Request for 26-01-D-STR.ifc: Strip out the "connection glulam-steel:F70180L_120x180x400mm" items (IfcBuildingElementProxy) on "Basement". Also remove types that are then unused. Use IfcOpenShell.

First a look at what the model holds.

```python
import ifcopenshell
import ifcopenshell.util.element

model = ifcopenshell.open("26-01-D-STR.ifc")
print(model.schema)
storey = next(s for s in model.by_type("IfcBuildingStorey") if s.Name == "Basement")
proxies = [e for e in ifcopenshell.util.element.get_decomposition(storey) if e.is_a("IfcBuildingElementProxy")]
seen = {}
for e in proxies:
    element_type = ifcopenshell.util.element.get_type(e)
    name = element_type.Name if element_type not in (None, e) else None
    seen[name] = seen.get(name, 0) + 1
for name, count in sorted(seen.items(), key=str):
    print(count, "x", name)
```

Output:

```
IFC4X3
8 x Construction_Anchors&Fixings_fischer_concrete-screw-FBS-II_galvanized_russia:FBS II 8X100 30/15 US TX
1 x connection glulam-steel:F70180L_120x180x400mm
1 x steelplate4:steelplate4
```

```python
import ifcopenshell
import ifcopenshell.api.root
import ifcopenshell.util.element

model = ifcopenshell.open("26-01-D-STR.ifc")

storey = next(s for s in model.by_type("IfcBuildingStorey") if s.Name == "Basement")
proxies = [e for e in ifcopenshell.util.element.get_decomposition(storey) if e.is_a("IfcBuildingElementProxy")]
targets = [e for e in proxies if (t := ifcopenshell.util.element.get_type(e)) not in (None, e) and t.Name == "connection glulam-steel:F70180L_120x180x400mm"]
types = {ifcopenshell.util.element.get_type(e) for e in targets} - {None, *targets}

for e in targets:
    ifcopenshell.api.root.remove_product(model, product=e)
print(len(targets), "removed")

unused = [t for t in types if not ifcopenshell.util.element.get_types(t)]
for t in unused:
    ifcopenshell.api.root.remove_product(model, product=t)
print(len(unused), "unused types removed")

model.write("26-01-D-STR_v2.ifc")
```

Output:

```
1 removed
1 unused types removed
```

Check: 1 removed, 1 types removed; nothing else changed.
